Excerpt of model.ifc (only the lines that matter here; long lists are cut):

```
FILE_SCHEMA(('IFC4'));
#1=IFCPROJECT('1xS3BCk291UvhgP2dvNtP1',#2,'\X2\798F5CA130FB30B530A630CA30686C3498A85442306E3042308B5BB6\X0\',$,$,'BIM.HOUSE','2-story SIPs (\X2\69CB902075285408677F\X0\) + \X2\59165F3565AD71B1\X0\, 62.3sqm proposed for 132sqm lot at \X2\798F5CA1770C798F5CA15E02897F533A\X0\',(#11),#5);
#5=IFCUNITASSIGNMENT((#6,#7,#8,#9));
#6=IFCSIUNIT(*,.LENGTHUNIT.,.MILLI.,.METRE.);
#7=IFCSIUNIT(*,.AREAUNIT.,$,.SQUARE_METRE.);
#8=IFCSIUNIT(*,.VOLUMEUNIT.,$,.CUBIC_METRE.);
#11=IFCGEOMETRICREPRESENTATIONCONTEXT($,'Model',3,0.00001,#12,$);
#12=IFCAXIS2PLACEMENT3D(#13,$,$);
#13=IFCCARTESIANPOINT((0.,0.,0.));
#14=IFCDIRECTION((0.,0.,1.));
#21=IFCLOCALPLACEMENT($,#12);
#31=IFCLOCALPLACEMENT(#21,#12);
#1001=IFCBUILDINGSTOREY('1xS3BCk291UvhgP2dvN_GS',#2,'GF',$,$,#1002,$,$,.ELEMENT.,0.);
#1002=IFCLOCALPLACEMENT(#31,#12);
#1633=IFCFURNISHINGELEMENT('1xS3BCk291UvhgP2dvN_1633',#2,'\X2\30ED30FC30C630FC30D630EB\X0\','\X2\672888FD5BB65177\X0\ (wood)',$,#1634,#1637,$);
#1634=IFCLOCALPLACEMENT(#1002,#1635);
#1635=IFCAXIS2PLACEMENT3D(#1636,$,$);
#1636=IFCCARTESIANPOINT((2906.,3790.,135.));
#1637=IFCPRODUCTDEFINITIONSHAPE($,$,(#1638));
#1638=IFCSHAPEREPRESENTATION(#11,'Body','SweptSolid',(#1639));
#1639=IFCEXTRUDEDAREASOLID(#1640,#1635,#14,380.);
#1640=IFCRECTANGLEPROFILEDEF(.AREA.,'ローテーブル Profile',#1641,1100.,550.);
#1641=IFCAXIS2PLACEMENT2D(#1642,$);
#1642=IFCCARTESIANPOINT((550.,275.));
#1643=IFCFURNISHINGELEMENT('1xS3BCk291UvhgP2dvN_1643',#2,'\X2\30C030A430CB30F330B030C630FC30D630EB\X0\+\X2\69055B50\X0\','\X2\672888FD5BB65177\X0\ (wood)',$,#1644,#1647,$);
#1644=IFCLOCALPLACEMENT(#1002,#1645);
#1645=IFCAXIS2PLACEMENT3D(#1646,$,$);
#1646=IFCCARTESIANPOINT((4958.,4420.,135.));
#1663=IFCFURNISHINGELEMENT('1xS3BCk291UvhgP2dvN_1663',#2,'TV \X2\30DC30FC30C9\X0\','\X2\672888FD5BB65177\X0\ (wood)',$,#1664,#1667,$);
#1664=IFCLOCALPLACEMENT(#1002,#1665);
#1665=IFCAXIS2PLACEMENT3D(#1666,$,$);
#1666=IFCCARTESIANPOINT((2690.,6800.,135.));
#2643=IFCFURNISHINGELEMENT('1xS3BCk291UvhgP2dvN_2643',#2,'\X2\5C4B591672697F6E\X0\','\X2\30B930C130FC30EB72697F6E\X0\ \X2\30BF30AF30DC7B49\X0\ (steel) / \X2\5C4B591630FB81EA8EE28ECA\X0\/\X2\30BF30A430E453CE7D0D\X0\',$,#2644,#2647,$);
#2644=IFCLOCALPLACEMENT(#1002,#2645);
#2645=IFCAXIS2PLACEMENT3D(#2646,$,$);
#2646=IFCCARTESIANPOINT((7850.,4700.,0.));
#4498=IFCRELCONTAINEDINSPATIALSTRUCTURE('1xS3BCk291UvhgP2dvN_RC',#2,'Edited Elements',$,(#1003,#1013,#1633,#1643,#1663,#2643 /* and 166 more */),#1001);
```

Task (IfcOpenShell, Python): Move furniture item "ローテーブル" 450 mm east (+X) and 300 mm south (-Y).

```python
import ifcopenshell
import ifcopenshell.api.geometry
import ifcopenshell.util.placement
import ifcopenshell.util.unit

model = ifcopenshell.open("model.ifc")
unit_scale = ifcopenshell.util.unit.calculate_unit_scale(model)

item = model.by_guid("1xS3BCk291UvhgP2dvN_1633")
matrix = ifcopenshell.util.placement.get_local_placement(item.ObjectPlacement)
matrix[0, 3] += 0.45 / unit_scale
matrix[1, 3] -= 0.3 / unit_scale
ifcopenshell.api.geometry.edit_object_placement(model, product=item, matrix=matrix, is_si=False)

print(ifcopenshell.util.placement.get_local_placement(item.ObjectPlacement).round(3) + 0.0)

model.write("model-out.ifc")
```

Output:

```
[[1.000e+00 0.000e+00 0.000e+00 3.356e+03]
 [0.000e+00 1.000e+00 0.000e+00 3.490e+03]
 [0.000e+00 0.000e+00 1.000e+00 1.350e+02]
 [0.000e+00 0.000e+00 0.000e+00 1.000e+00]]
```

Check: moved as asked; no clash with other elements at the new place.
